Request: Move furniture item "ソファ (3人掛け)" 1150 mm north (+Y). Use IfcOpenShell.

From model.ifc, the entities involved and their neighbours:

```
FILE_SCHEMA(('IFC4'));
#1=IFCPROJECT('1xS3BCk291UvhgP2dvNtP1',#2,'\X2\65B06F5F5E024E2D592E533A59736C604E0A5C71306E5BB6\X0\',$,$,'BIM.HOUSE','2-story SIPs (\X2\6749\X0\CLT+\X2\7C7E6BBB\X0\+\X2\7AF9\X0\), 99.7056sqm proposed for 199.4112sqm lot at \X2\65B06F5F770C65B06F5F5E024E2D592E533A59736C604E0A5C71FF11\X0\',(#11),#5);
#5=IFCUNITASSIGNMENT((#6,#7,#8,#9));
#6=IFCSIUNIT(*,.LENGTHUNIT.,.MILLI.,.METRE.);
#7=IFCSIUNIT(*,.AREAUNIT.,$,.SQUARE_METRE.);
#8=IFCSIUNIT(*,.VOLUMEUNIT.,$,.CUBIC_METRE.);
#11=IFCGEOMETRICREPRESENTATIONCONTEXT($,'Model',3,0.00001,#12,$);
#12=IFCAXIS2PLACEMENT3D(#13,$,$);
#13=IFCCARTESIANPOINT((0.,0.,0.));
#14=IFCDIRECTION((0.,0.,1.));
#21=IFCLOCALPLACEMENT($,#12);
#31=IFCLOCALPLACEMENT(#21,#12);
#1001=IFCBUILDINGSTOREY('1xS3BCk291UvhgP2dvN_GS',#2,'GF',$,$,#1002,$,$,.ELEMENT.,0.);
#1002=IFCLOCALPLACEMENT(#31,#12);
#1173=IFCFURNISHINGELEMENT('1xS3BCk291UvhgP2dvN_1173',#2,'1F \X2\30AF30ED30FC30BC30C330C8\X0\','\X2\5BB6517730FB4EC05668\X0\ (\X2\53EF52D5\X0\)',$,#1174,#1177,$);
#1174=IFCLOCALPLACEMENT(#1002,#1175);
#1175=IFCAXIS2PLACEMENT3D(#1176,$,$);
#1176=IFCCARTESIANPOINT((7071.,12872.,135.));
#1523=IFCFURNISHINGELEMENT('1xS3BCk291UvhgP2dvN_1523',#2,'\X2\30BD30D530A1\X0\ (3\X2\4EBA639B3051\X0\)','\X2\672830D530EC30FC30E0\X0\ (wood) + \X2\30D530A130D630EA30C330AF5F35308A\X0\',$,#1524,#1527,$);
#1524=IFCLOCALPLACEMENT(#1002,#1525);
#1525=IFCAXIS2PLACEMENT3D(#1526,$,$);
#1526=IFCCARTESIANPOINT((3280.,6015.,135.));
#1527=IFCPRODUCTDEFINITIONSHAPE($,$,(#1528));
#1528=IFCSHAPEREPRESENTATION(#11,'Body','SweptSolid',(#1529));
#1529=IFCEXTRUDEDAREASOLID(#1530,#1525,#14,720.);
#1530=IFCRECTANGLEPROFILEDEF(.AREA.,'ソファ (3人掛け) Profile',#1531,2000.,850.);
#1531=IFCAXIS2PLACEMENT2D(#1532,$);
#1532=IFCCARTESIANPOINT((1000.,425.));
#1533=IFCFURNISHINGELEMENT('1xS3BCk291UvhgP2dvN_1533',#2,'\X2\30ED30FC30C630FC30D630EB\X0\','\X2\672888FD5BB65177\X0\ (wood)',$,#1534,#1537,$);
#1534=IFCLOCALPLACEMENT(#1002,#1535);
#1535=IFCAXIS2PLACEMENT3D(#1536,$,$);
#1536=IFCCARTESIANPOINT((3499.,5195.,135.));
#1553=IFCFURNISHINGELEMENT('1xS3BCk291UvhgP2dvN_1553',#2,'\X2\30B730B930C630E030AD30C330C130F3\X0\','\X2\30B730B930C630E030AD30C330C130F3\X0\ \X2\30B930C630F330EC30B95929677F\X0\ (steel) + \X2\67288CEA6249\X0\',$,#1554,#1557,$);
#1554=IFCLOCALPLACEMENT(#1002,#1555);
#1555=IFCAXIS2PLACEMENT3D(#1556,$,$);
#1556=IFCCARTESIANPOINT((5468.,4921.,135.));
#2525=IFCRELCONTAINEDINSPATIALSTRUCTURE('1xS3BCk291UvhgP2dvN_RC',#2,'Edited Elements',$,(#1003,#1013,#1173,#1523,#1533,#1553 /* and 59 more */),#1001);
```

```python
import ifcopenshell
import ifcopenshell.api.geometry
import ifcopenshell.util.placement

model = ifcopenshell.open("model.ifc")

item = model.by_guid("1xS3BCk291UvhgP2dvN_1523")
matrix = ifcopenshell.util.placement.get_local_placement(item.ObjectPlacement)
matrix[1, 3] += 1150.0
ifcopenshell.api.geometry.edit_object_placement(model, product=item, matrix=matrix, is_si=False)

print(ifcopenshell.util.placement.get_local_placement(item.ObjectPlacement).round(3) + 0.0)

model.write("model-out.ifc")
```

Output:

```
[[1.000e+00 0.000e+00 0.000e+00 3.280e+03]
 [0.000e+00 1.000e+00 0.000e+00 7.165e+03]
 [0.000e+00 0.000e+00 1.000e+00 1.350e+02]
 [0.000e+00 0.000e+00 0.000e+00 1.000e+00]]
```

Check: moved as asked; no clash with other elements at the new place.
